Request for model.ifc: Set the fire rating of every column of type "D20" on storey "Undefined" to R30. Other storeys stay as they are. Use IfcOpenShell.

First a look at what the model holds.

```python
import ifcopenshell
import ifcopenshell.util.element

model = ifcopenshell.open("model.ifc")
print(model.schema)
storey = next(s for s in model.by_type("IfcBuildingStorey") if s.Name == "Undefined")
columns = [e for e in ifcopenshell.util.element.get_decomposition(storey) if e.is_a("IfcColumn")]
seen = {}
for e in columns:
    element_type = ifcopenshell.util.element.get_type(e)
    key = (element_type.Name if element_type != e and element_type else None, ifcopenshell.util.element.get_pset(e, "Pset_ColumnCommon", "FireRating"))
    seen[key] = seen.get(key, 0) + 1
for (name, value), count in sorted(seen.items(), key=str):
    print(count, "x", name, "|", value)
```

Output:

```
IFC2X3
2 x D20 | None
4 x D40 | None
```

```python
import ifcopenshell
import ifcopenshell.api.pset
import ifcopenshell.util.element

model = ifcopenshell.open("model.ifc")

storey = next(s for s in model.by_type("IfcBuildingStorey") if s.Name == "Undefined")
columns = [e for e in ifcopenshell.util.element.get_decomposition(storey) if e.is_a("IfcColumn")]

count = 0
for e in columns:
    element_type = ifcopenshell.util.element.get_type(e)
    if element_type in (None, e) or element_type.Name != "D20":
        continue
    found = ifcopenshell.util.element.get_pset(e, "Pset_ColumnCommon", should_inherit=False)
    if found:
        pset = model.by_id(found["id"])
        if len(ifcopenshell.util.element.get_elements_by_pset(pset)) > 1:
            pset = ifcopenshell.api.pset.unshare_pset(model, products=[e], pset=pset)[0]
    else:
        pset = ifcopenshell.api.pset.add_pset(model, product=e, name="Pset_ColumnCommon")
    ifcopenshell.api.pset.edit_pset(model, pset=pset, properties={"FireRating": "R30"})
    count += 1

print(count, "columns updated")

model.write("model_v2.ifc")
```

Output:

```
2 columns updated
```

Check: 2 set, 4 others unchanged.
